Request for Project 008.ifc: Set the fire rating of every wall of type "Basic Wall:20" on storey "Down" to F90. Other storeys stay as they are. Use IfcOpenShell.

First a look at what the model holds.

```python
import ifcopenshell
import ifcopenshell.util.element

model = ifcopenshell.open("Project 008.ifc")
print(model.schema)
storey = next(s for s in model.by_type("IfcBuildingStorey") if s.Name == "Down")
walls = [e for e in ifcopenshell.util.element.get_decomposition(storey) if e.is_a("IfcWall")]
seen = {}
for e in walls:
    element_type = ifcopenshell.util.element.get_type(e)
    key = (element_type.Name if element_type != e and element_type else None, ifcopenshell.util.element.get_pset(e, "Pset_WallCommon", "FireRating"))
    seen[key] = seen.get(key, 0) + 1
for (name, value), count in sorted(seen.items(), key=str):
    print(count, "x", name, "|", value)
```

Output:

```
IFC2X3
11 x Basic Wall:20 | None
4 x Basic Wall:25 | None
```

```python
import ifcopenshell
import ifcopenshell.api.pset
import ifcopenshell.util.element

model = ifcopenshell.open("Project 008.ifc")

storey = next(s for s in model.by_type("IfcBuildingStorey") if s.Name == "Down")
walls = [e for e in ifcopenshell.util.element.get_decomposition(storey) if e.is_a("IfcWall")]

count = 0
for e in walls:
    element_type = ifcopenshell.util.element.get_type(e)
    if element_type in (None, e) or element_type.Name != "Basic Wall:20":
        continue
    # add_pset returns the element's existing set when there is one.
    pset = ifcopenshell.api.pset.add_pset(model, product=e, name="Pset_WallCommon")
    ifcopenshell.api.pset.edit_pset(model, pset=pset, properties={"FireRating": "F90"})
    count += 1

print(count, "walls updated")

model.write("Project 008-out.ifc")
```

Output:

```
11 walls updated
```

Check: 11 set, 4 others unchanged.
